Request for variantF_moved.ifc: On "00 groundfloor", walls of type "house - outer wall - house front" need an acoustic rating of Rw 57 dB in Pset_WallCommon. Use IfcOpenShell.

First a look at what the model holds.

```python
import ifcopenshell
import ifcopenshell.util.element

model = ifcopenshell.open("variantF_moved.ifc")
print(model.schema)
storey = next(s for s in model.by_type("IfcBuildingStorey") if s.Name == "00 groundfloor")
walls = [e for e in ifcopenshell.util.element.get_decomposition(storey) if e.is_a("IfcWall")]
seen = {}
for e in walls:
    element_type = ifcopenshell.util.element.get_type(e)
    key = (element_type.Name if element_type != e and element_type else None, ifcopenshell.util.element.get_pset(e, "Pset_WallCommon", "AcousticRating"))
    seen[key] = seen.get(key, 0) + 1
for (name, value), count in sorted(seen.items(), key=str):
    print(count, "x", name, "|", value)
```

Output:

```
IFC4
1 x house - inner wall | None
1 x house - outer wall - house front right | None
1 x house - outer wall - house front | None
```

```python
import ifcopenshell
import ifcopenshell.api.pset
import ifcopenshell.util.element

model = ifcopenshell.open("variantF_moved.ifc")

storey = next(s for s in model.by_type("IfcBuildingStorey") if s.Name == "00 groundfloor")
walls = [e for e in ifcopenshell.util.element.get_decomposition(storey) if e.is_a("IfcWall")]

count = 0
for e in walls:
    element_type = ifcopenshell.util.element.get_type(e)
    if element_type in (None, e) or element_type.Name != "house - outer wall - house front":
        continue
    # add_pset returns the element's existing set when there is one.
    pset = ifcopenshell.api.pset.add_pset(model, product=e, name="Pset_WallCommon")
    ifcopenshell.api.pset.edit_pset(model, pset=pset, properties={"AcousticRating": "Rw 57 dB"})
    count += 1

print(count, "walls updated")

model.write("variantF_moved_updated.ifc")
```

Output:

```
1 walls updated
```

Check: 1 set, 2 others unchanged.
